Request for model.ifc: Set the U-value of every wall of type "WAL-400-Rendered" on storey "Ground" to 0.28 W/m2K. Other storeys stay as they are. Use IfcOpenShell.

First a look at what the model holds.

```python
import ifcopenshell
import ifcopenshell.util.element

model = ifcopenshell.open("model.ifc")
print(model.schema)
storey = next(s for s in model.by_type("IfcBuildingStorey") if s.Name == "Ground")
walls = [e for e in ifcopenshell.util.element.get_decomposition(storey) if e.is_a("IfcWall")]
seen = {}
for e in walls:
    element_type = ifcopenshell.util.element.get_type(e)
    key = (element_type.Name if element_type != e and element_type else None, ifcopenshell.util.element.get_pset(e, "Pset_WallCommon", "ThermalTransmittance"))
    seen[key] = seen.get(key, 0) + 1
for (name, value), count in sorted(seen.items(), key=str):
    print(count, "x", name, "|", value)
```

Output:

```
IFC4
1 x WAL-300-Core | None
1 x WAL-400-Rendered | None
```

```python
import ifcopenshell
import ifcopenshell.api.pset
import ifcopenshell.util.element

model = ifcopenshell.open("model.ifc")

storey = next(s for s in model.by_type("IfcBuildingStorey") if s.Name == "Ground")
walls = [e for e in ifcopenshell.util.element.get_decomposition(storey) if e.is_a("IfcWall")]

count = 0
for e in walls:
    element_type = ifcopenshell.util.element.get_type(e)
    if element_type in (None, e) or element_type.Name != "WAL-400-Rendered":
        continue
    # add_pset returns the element's existing set when there is one.
    pset = ifcopenshell.api.pset.add_pset(model, product=e, name="Pset_WallCommon")
    ifcopenshell.api.pset.edit_pset(model, pset=pset, properties={"ThermalTransmittance": 0.28})
    count += 1

print(count, "walls updated")

model.write("model_v2.ifc")
```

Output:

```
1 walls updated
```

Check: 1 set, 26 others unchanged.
